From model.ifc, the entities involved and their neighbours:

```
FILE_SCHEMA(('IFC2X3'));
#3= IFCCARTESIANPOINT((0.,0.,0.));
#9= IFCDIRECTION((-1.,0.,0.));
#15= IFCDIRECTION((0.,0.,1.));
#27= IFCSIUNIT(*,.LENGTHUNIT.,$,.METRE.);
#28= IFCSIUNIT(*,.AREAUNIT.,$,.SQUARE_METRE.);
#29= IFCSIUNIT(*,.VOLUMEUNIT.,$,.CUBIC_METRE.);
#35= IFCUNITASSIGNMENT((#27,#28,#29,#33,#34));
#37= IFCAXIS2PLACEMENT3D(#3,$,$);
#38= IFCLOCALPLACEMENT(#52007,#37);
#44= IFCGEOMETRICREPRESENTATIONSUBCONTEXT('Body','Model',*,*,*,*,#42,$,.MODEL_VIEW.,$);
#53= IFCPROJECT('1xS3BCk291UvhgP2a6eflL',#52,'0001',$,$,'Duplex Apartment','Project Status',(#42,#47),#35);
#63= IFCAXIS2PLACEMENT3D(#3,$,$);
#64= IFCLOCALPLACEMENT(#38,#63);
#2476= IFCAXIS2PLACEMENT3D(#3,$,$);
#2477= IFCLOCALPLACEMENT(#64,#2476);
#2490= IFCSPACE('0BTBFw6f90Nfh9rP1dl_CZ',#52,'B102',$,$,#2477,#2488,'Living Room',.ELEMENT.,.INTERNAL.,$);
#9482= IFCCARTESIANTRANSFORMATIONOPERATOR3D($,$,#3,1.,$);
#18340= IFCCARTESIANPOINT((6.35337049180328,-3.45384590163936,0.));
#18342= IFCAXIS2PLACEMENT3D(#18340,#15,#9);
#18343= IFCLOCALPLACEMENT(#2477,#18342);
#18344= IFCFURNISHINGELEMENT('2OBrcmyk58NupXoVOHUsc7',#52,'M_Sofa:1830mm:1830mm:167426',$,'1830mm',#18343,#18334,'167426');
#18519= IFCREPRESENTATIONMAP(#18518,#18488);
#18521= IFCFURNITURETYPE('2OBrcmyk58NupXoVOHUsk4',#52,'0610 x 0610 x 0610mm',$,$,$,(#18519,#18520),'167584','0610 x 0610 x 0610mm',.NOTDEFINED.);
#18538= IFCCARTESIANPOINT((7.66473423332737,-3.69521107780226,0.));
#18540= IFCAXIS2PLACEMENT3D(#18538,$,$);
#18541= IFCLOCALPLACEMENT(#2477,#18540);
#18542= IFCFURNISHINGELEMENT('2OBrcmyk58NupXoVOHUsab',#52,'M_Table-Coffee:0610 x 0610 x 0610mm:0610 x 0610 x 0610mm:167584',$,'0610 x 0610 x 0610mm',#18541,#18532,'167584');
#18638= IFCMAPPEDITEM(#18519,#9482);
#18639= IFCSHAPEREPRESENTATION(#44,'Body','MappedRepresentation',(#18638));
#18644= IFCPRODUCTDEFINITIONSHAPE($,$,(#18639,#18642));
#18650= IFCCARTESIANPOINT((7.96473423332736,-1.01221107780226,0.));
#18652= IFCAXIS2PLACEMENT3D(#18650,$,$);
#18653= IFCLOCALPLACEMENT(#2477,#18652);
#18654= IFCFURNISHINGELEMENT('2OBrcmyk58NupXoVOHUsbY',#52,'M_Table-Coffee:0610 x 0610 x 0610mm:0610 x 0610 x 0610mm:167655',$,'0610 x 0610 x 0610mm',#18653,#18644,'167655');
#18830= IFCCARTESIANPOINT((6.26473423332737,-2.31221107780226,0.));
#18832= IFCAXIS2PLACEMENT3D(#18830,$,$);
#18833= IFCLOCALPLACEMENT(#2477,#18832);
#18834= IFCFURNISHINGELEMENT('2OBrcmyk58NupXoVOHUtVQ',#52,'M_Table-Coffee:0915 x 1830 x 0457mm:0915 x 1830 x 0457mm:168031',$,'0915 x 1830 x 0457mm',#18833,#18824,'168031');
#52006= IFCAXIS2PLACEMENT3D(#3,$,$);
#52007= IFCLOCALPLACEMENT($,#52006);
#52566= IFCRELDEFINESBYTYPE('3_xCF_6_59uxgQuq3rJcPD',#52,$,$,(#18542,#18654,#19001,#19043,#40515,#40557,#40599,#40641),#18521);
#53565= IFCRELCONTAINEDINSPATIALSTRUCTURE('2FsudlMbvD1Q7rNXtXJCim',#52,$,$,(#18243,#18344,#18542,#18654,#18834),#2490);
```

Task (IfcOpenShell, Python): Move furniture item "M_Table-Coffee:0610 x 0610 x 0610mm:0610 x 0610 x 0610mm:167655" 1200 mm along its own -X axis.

```python
import ifcopenshell
import ifcopenshell.api.geometry
import ifcopenshell.util.placement

model = ifcopenshell.open("model.ifc")

item = model.by_id(18654)
matrix = ifcopenshell.util.placement.get_local_placement(item.ObjectPlacement)
matrix[:3, 3] -= matrix[:3, 0] * 1.2
ifcopenshell.api.geometry.edit_object_placement(model, product=item, matrix=matrix, is_si=False)

print(ifcopenshell.util.placement.get_local_placement(item.ObjectPlacement).round(3) + 0.0)

model.write("model_rev.ifc")
```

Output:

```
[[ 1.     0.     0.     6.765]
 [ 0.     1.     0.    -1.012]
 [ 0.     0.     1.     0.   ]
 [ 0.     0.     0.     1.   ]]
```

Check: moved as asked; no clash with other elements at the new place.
